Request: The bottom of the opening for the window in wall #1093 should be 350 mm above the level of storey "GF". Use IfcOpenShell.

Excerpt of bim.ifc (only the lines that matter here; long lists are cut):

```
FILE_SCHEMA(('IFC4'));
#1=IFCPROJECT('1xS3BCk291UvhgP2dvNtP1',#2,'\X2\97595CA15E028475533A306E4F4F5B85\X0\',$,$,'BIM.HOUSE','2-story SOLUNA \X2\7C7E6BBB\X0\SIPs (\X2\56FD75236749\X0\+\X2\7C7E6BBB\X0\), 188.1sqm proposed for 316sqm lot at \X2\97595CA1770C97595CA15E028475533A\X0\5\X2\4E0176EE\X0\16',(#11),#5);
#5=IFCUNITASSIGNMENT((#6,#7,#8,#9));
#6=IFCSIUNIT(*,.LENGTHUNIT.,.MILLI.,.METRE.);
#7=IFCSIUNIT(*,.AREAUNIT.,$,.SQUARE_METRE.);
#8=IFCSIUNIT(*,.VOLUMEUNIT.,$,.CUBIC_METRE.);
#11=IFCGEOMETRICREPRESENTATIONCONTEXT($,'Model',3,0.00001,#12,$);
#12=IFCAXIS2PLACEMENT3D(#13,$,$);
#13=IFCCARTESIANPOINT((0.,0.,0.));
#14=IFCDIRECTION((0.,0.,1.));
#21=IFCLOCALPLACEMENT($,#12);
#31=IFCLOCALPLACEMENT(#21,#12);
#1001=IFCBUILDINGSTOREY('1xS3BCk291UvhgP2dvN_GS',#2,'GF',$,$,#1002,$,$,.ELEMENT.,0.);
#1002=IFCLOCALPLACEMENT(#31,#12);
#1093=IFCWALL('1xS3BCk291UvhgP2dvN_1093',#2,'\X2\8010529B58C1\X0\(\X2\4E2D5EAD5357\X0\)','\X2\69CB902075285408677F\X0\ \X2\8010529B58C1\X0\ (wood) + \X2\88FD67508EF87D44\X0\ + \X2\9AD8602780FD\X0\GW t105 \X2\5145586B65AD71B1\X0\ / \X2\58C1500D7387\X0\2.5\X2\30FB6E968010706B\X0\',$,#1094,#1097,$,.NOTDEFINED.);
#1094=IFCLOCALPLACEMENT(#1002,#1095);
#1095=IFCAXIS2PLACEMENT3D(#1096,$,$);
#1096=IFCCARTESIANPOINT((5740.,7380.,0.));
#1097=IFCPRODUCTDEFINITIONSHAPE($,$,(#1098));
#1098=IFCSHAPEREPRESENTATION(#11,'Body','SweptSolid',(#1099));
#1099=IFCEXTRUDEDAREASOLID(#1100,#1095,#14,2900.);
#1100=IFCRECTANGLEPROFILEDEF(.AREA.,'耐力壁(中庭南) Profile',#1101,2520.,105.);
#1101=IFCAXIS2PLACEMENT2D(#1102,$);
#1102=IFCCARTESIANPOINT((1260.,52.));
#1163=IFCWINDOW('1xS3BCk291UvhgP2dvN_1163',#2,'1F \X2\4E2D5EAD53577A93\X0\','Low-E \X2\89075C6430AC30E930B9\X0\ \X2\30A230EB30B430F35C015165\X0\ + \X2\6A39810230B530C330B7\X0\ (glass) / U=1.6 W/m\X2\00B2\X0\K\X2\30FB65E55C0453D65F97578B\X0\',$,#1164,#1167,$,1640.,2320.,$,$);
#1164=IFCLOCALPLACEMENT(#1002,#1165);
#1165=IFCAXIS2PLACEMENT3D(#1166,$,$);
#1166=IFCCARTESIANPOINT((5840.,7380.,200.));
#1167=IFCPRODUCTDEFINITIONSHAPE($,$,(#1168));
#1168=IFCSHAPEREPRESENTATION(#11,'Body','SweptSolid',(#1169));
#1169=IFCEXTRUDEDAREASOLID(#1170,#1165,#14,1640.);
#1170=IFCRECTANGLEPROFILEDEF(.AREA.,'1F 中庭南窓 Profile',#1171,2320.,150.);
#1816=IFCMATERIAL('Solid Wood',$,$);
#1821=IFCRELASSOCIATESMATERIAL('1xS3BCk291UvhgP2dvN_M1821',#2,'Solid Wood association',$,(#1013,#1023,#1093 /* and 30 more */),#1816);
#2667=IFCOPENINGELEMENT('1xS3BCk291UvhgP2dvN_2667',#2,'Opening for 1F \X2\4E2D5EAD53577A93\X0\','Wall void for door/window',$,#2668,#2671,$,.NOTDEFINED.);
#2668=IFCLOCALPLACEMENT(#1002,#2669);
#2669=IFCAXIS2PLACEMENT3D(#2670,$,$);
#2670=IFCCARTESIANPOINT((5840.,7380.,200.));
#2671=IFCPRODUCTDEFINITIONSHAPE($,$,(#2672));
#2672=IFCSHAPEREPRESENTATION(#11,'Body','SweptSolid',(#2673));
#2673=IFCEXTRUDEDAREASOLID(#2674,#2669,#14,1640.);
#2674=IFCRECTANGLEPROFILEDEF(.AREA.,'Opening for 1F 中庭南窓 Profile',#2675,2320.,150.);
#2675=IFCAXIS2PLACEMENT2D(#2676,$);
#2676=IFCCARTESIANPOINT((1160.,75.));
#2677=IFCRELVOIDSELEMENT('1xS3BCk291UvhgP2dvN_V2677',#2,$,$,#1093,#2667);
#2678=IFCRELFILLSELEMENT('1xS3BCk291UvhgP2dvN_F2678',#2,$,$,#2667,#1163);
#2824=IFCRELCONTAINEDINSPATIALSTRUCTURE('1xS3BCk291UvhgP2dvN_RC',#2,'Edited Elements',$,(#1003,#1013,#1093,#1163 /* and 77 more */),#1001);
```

```python
import numpy as np
import ifcopenshell
import ifcopenshell.api.geometry
import ifcopenshell.geom
import ifcopenshell.util.element
import ifcopenshell.util.placement
import ifcopenshell.util.shape
import ifcopenshell.util.unit

model = ifcopenshell.open("bim.ifc")
unit_scale = ifcopenshell.util.unit.calculate_unit_scale(model)

window = model.by_guid("1xS3BCk291UvhgP2dvN_1163")
opening = window.FillsVoids[0].RelatingOpeningElement
storey = ifcopenshell.util.element.get_container(window, ifc_class="IfcBuildingStorey")
level = ifcopenshell.util.placement.get_local_placement(storey.ObjectPlacement)[2, 3]

# The opening's origin need not be at the sill, so measure its lowest point.
shape = ifcopenshell.geom.create_shape(ifcopenshell.geom.settings(), opening)
bottom = ifcopenshell.util.shape.get_shape_bottom_elevation(shape, shape.geometry) / unit_scale
dz = level + 0.35 / unit_scale - bottom

shift = np.array([0.0, 0.0, dz])
# The window is not placed relative to its opening, so move both.
for product in (opening, window):
    matrix = ifcopenshell.util.placement.get_local_placement(product.ObjectPlacement)
    matrix[:3, 3] += shift
    ifcopenshell.api.geometry.edit_object_placement(model, product=product, matrix=matrix, is_si=False)

print(f"moved by {dz * unit_scale:+.3f} m")

model.write("bim_v2.ifc")
```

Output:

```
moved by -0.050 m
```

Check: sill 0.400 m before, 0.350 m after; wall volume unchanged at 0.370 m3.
